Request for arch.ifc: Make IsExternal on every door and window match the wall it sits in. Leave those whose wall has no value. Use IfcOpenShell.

First a look at what the model holds.

```python
import ifcopenshell
import ifcopenshell.util.element

model = ifcopenshell.open("arch.ifc")
print(model.schema)
seen = {}
for e in model.by_type("IfcDoor") + model.by_type("IfcWindow"):
    if not e.FillsVoids:
        continue
    host = e.FillsVoids[0].RelatingOpeningElement.VoidsElements[0].RelatingBuildingElement
    own = ifcopenshell.util.element.get_pset(e, f"Pset_{e.is_a()[3:].removesuffix('StandardCase')}Common", "IsExternal")
    wall = ifcopenshell.util.element.get_pset(host, "Pset_WallCommon", "IsExternal")
    seen[e.is_a(), own, wall] = seen.get((e.is_a(), own, wall), 0) + 1
for (cls, own, wall), count in sorted(seen.items(), key=str):
    print(count, cls, "IsExternal:", own, "| host wall:", wall)
```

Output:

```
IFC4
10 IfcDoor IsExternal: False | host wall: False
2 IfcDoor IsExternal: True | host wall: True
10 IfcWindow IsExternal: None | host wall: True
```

```python
import ifcopenshell
import ifcopenshell.api.pset
import ifcopenshell.util.element

model = ifcopenshell.open("arch.ifc")

count = 0
for ifc_class, pset_name in (("IfcDoor", "Pset_DoorCommon"), ("IfcWindow", "Pset_WindowCommon")):
    for e in model.by_type(ifc_class):
        if not e.FillsVoids:
            continue
        host = e.FillsVoids[0].RelatingOpeningElement.VoidsElements[0].RelatingBuildingElement
        external = ifcopenshell.util.element.get_pset(host, "Pset_WallCommon", "IsExternal")
        if external is None or ifcopenshell.util.element.get_pset(e, pset_name, "IsExternal") == external:
            continue
        pset = ifcopenshell.api.pset.add_pset(model, product=e, name=pset_name)
        ifcopenshell.api.pset.edit_pset(model, pset=pset, properties={"IsExternal": external})
        count += 1

print(count, "updated")

model.write("arch_rev.ifc")
```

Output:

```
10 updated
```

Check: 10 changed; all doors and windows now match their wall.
